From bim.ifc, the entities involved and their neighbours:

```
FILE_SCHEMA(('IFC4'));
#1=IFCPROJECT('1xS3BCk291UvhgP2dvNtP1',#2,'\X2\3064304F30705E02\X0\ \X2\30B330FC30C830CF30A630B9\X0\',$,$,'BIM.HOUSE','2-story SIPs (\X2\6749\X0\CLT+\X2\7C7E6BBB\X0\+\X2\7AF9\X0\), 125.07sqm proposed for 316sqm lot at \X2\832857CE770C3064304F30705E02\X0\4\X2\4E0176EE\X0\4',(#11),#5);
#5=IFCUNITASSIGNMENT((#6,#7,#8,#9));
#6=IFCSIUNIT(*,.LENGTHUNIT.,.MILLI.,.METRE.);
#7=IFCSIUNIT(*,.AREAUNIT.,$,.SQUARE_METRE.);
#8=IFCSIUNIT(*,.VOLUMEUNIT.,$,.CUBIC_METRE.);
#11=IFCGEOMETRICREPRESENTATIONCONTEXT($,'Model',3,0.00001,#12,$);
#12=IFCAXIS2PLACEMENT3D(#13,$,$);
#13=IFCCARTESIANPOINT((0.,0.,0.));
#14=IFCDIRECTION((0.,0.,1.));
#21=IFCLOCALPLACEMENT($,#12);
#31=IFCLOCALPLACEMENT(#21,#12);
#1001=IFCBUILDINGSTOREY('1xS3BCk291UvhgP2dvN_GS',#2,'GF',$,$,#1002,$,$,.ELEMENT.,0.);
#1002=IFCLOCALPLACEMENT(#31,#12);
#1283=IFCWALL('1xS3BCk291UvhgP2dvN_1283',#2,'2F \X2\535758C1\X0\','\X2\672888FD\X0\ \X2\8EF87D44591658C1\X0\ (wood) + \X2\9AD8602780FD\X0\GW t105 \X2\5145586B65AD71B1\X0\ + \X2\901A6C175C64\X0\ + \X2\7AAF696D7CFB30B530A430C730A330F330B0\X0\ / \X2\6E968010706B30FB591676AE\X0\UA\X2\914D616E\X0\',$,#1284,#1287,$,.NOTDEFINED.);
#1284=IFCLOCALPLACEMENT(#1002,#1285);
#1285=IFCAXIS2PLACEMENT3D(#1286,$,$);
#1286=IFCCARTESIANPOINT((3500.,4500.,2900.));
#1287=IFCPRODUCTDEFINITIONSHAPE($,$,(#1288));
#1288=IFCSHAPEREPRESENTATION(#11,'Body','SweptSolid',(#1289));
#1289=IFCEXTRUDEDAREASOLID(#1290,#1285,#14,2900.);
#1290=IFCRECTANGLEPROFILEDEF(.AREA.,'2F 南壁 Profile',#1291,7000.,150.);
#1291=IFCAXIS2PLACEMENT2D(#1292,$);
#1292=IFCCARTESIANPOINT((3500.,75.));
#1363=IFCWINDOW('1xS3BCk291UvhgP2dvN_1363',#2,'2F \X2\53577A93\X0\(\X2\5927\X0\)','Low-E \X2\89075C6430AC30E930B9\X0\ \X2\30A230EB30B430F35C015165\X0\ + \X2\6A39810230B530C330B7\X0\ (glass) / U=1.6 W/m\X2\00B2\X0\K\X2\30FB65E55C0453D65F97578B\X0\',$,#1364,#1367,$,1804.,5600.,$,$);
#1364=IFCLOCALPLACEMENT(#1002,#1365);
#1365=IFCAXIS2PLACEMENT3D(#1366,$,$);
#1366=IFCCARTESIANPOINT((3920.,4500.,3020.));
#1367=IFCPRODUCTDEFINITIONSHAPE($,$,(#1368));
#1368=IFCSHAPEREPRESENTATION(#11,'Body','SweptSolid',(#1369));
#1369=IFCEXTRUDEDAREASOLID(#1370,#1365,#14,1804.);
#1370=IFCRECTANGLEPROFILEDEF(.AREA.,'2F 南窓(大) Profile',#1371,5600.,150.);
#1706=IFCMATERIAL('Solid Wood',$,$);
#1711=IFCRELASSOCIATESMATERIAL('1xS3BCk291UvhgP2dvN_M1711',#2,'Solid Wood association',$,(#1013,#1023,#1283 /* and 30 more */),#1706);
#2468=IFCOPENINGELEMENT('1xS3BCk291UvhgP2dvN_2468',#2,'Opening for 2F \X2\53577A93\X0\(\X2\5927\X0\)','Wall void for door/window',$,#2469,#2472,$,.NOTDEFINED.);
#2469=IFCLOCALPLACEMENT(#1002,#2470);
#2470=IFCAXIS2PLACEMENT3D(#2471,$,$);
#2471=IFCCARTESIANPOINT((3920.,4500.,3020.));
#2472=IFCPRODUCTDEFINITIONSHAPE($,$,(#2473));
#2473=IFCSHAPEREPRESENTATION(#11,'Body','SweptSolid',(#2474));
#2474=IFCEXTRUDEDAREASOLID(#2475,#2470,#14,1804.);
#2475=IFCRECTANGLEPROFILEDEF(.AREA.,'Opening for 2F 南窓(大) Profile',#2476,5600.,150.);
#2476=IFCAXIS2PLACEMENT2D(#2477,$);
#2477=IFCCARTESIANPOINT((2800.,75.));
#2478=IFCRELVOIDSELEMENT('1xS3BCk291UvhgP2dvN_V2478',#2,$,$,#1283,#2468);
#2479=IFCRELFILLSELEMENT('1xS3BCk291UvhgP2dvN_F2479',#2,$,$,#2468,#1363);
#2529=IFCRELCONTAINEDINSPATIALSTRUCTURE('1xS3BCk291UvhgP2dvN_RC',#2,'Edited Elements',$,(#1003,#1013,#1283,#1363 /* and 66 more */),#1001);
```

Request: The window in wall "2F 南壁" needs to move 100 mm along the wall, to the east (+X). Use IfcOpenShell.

```python
import ifcopenshell
import ifcopenshell.api.geometry
import ifcopenshell.util.placement
import ifcopenshell.util.unit

model = ifcopenshell.open("bim.ifc")
unit_scale = ifcopenshell.util.unit.calculate_unit_scale(model)

window = model.by_guid("1xS3BCk291UvhgP2dvN_1363")
opening = window.FillsVoids[0].RelatingOpeningElement
wall = opening.VoidsElements[0].RelatingBuildingElement

wall_matrix = ifcopenshell.util.placement.get_local_placement(wall.ObjectPlacement)
shift = wall_matrix[:3, 0] * 0.1 / unit_scale
before = ifcopenshell.util.placement.get_local_placement(window.ObjectPlacement)[:3, 3].copy()

# The window is not placed relative to its opening, so move both.
for product in (opening, window):
    matrix = ifcopenshell.util.placement.get_local_placement(product.ObjectPlacement)
    matrix[:3, 3] += shift
    ifcopenshell.api.geometry.edit_object_placement(model, product=product, matrix=matrix, is_si=False)

after = ifcopenshell.util.placement.get_local_placement(window.ObjectPlacement)[:3, 3]
print("window moved by", (after - before).round(3) + 0.0)

model.write("bim-out.ifc")
```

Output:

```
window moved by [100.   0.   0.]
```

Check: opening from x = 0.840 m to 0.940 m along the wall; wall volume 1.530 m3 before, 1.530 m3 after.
